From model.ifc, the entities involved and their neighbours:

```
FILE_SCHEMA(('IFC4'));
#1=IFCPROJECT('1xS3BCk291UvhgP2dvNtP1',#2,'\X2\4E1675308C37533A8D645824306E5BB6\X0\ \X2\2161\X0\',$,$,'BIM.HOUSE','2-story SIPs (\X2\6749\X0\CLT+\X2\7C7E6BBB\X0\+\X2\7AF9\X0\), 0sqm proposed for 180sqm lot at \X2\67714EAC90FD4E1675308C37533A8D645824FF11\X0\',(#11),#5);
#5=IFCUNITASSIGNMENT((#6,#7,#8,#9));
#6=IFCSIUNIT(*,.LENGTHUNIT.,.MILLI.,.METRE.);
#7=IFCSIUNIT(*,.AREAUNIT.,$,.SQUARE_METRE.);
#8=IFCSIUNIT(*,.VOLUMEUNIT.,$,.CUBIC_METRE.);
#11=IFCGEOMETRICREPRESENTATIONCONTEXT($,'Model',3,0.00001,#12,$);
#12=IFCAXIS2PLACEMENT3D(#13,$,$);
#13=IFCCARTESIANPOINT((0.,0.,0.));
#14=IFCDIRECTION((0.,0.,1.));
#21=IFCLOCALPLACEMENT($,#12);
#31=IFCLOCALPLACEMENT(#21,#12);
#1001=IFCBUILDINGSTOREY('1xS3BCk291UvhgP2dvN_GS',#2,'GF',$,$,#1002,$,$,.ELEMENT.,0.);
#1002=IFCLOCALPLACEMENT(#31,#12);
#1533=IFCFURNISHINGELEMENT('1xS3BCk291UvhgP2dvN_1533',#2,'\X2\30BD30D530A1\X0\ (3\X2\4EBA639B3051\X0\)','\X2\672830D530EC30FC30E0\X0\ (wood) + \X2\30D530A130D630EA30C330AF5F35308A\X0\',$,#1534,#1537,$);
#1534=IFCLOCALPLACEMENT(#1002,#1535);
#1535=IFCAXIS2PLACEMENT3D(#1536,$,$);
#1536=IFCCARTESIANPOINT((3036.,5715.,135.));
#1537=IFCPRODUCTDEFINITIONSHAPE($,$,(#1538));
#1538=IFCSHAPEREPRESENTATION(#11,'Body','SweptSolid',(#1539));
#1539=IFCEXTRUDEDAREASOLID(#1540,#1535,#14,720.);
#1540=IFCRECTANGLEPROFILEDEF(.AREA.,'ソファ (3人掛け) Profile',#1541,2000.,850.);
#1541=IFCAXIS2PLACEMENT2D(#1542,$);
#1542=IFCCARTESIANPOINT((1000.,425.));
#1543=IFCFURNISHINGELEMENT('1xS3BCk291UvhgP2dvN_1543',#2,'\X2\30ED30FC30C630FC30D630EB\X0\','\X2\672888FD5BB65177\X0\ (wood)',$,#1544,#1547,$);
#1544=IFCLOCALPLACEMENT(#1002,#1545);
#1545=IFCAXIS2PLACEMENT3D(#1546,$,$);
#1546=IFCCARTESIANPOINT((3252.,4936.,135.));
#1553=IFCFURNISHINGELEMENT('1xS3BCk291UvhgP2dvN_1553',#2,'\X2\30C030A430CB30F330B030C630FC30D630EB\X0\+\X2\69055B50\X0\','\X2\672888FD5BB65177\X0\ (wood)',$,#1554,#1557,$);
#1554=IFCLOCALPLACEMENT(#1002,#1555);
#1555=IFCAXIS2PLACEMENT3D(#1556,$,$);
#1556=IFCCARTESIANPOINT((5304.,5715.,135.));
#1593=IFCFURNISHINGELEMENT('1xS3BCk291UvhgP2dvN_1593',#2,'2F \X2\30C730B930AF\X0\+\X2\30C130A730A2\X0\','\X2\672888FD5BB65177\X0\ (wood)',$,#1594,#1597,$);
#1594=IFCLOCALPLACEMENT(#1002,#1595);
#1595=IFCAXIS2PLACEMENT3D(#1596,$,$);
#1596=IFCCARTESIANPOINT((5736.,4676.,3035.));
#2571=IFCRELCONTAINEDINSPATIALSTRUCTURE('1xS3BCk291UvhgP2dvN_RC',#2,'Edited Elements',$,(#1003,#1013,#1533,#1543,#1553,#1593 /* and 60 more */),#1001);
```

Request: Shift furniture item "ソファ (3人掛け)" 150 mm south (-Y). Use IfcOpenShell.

```python
import ifcopenshell
import ifcopenshell.api.geometry
import ifcopenshell.util.placement

model = ifcopenshell.open("model.ifc")

item = model.by_guid("1xS3BCk291UvhgP2dvN_1533")
matrix = ifcopenshell.util.placement.get_local_placement(item.ObjectPlacement)
matrix[1, 3] -= 150.0
ifcopenshell.api.geometry.edit_object_placement(model, product=item, matrix=matrix, is_si=False)

print(ifcopenshell.util.placement.get_local_placement(item.ObjectPlacement).round(3) + 0.0)

model.write("model_rev.ifc")
```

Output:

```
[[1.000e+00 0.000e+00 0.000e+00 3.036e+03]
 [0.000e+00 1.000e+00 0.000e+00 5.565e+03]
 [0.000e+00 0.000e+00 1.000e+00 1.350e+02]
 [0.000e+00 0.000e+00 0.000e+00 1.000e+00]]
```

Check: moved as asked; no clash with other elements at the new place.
